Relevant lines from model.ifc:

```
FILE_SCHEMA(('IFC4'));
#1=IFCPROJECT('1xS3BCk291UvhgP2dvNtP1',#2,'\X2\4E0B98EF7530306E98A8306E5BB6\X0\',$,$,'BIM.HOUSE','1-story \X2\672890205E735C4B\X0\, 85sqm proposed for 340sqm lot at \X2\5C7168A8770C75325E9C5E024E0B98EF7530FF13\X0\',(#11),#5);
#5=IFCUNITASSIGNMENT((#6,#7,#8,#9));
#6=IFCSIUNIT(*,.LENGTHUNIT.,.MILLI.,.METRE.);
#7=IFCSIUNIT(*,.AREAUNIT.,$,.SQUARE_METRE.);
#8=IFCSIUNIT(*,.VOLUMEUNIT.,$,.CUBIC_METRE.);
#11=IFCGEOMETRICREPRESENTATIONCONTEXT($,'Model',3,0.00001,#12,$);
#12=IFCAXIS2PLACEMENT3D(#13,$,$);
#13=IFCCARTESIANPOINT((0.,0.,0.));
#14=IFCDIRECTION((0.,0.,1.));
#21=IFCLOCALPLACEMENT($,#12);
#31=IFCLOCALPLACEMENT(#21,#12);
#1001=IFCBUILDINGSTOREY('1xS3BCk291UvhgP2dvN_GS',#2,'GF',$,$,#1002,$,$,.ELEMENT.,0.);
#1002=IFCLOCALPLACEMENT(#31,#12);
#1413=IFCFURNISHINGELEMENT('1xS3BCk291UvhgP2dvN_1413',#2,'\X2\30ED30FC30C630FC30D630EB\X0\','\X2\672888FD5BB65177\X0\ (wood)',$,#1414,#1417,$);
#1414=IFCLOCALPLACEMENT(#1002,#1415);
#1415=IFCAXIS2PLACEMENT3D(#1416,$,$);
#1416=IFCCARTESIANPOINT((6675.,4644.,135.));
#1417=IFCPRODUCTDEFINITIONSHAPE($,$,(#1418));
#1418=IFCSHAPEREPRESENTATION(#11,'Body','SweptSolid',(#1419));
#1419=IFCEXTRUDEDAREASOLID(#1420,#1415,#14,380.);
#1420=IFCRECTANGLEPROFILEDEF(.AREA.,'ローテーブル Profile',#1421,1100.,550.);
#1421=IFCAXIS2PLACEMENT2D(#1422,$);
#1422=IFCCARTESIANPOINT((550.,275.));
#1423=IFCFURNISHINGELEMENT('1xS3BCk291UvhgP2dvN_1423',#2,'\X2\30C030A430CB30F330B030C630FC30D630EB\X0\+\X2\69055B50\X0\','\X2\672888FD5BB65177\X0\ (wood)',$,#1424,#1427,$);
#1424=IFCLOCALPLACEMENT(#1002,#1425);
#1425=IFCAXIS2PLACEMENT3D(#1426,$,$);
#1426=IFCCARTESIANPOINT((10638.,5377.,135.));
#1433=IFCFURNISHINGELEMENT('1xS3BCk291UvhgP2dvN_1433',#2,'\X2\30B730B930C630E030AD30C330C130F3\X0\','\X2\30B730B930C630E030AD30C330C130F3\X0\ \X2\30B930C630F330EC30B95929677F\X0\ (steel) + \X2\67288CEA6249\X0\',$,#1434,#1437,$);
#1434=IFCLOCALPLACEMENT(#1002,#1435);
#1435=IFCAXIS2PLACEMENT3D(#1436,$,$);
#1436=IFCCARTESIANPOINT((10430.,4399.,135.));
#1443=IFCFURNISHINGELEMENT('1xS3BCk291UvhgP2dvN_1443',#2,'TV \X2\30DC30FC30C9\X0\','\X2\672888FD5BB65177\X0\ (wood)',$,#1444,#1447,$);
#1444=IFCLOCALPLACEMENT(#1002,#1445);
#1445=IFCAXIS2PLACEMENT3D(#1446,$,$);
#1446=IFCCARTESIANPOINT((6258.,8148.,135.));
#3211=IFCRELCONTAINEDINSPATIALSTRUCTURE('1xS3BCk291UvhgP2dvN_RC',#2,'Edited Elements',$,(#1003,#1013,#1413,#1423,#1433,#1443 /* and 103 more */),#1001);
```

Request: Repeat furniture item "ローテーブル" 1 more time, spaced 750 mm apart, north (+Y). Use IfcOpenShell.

```python
import numpy as np
import ifcopenshell
import ifcopenshell.api.geometry
import ifcopenshell.api.root
import ifcopenshell.util.element
import ifcopenshell.util.placement

model = ifcopenshell.open("model.ifc")


def reuse_history(source, copy):
    """copy_class also copies each property set's owner history, people and application; keep the originals."""
    for rel in copy.IsDefinedBy:
        if rel.is_a("IfcRelDefinesByProperties") and (history := rel.RelatingPropertyDefinition.OwnerHistory):
            rel.RelatingPropertyDefinition.OwnerHistory = source.OwnerHistory
            ifcopenshell.util.element.remove_deep2(model, history)


source = model.by_guid("1xS3BCk291UvhgP2dvN_1413")
base = ifcopenshell.util.placement.get_local_placement(source.ObjectPlacement)
step = np.array([0.0, 1.0, 0.0]) * 750.0

for i in range(1, 2):
    copy = ifcopenshell.api.root.copy_class(model, product=source)
    copy.Representation = ifcopenshell.util.element.copy_deep(
        model, source.Representation, exclude=["IfcGeometricRepresentationContext", "IfcRepresentationMap"]
    )
    reuse_history(source, copy)
    matrix = base.copy()
    matrix[:3, 3] += i * step
    print("added at", matrix[:3, 3].round(3) + 0.0)
    ifcopenshell.api.geometry.edit_object_placement(model, product=copy, matrix=matrix, is_si=False)

model.write("model_edited.ifc")
```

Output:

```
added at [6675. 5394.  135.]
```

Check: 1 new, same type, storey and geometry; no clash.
